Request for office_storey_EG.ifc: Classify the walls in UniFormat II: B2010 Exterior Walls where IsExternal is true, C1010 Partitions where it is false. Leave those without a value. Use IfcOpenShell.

First a look at what the model holds.

```python
import ifcopenshell
import ifcopenshell.util.element

model = ifcopenshell.open("office_storey_EG.ifc")
print(model.schema)
print("classifications:", [c.Name for c in model.by_type("IfcClassification")])
values = [ifcopenshell.util.element.get_pset(e, "Pset_WallCommon", "IsExternal") for e in model.by_type("IfcWall")]
for value in (True, False, None):
    print("IsExternal", value, values.count(value))
```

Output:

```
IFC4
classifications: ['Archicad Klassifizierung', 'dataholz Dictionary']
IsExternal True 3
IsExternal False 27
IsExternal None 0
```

```python
import ifcopenshell
import ifcopenshell.api.classification
import ifcopenshell.util.element

model = ifcopenshell.open("office_storey_EG.ifc")

system = ifcopenshell.api.classification.add_classification(model, classification="UniFormat II")

walls = model.by_type("IfcWall")
external = {e: ifcopenshell.util.element.get_pset(e, "Pset_WallCommon", "IsExternal") for e in walls}
for flag, code, name in ((True, "B2010", "Exterior Walls"), (False, "C1010", "Partitions")):
    products = [e for e in walls if external[e] is flag]
    ifcopenshell.api.classification.add_reference(
        model, products=products, classification=system, identification=code, name=name
    )
    print(code, len(products))

model.write("office_storey_EG-out.ifc")
```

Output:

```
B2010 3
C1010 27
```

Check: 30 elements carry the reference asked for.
